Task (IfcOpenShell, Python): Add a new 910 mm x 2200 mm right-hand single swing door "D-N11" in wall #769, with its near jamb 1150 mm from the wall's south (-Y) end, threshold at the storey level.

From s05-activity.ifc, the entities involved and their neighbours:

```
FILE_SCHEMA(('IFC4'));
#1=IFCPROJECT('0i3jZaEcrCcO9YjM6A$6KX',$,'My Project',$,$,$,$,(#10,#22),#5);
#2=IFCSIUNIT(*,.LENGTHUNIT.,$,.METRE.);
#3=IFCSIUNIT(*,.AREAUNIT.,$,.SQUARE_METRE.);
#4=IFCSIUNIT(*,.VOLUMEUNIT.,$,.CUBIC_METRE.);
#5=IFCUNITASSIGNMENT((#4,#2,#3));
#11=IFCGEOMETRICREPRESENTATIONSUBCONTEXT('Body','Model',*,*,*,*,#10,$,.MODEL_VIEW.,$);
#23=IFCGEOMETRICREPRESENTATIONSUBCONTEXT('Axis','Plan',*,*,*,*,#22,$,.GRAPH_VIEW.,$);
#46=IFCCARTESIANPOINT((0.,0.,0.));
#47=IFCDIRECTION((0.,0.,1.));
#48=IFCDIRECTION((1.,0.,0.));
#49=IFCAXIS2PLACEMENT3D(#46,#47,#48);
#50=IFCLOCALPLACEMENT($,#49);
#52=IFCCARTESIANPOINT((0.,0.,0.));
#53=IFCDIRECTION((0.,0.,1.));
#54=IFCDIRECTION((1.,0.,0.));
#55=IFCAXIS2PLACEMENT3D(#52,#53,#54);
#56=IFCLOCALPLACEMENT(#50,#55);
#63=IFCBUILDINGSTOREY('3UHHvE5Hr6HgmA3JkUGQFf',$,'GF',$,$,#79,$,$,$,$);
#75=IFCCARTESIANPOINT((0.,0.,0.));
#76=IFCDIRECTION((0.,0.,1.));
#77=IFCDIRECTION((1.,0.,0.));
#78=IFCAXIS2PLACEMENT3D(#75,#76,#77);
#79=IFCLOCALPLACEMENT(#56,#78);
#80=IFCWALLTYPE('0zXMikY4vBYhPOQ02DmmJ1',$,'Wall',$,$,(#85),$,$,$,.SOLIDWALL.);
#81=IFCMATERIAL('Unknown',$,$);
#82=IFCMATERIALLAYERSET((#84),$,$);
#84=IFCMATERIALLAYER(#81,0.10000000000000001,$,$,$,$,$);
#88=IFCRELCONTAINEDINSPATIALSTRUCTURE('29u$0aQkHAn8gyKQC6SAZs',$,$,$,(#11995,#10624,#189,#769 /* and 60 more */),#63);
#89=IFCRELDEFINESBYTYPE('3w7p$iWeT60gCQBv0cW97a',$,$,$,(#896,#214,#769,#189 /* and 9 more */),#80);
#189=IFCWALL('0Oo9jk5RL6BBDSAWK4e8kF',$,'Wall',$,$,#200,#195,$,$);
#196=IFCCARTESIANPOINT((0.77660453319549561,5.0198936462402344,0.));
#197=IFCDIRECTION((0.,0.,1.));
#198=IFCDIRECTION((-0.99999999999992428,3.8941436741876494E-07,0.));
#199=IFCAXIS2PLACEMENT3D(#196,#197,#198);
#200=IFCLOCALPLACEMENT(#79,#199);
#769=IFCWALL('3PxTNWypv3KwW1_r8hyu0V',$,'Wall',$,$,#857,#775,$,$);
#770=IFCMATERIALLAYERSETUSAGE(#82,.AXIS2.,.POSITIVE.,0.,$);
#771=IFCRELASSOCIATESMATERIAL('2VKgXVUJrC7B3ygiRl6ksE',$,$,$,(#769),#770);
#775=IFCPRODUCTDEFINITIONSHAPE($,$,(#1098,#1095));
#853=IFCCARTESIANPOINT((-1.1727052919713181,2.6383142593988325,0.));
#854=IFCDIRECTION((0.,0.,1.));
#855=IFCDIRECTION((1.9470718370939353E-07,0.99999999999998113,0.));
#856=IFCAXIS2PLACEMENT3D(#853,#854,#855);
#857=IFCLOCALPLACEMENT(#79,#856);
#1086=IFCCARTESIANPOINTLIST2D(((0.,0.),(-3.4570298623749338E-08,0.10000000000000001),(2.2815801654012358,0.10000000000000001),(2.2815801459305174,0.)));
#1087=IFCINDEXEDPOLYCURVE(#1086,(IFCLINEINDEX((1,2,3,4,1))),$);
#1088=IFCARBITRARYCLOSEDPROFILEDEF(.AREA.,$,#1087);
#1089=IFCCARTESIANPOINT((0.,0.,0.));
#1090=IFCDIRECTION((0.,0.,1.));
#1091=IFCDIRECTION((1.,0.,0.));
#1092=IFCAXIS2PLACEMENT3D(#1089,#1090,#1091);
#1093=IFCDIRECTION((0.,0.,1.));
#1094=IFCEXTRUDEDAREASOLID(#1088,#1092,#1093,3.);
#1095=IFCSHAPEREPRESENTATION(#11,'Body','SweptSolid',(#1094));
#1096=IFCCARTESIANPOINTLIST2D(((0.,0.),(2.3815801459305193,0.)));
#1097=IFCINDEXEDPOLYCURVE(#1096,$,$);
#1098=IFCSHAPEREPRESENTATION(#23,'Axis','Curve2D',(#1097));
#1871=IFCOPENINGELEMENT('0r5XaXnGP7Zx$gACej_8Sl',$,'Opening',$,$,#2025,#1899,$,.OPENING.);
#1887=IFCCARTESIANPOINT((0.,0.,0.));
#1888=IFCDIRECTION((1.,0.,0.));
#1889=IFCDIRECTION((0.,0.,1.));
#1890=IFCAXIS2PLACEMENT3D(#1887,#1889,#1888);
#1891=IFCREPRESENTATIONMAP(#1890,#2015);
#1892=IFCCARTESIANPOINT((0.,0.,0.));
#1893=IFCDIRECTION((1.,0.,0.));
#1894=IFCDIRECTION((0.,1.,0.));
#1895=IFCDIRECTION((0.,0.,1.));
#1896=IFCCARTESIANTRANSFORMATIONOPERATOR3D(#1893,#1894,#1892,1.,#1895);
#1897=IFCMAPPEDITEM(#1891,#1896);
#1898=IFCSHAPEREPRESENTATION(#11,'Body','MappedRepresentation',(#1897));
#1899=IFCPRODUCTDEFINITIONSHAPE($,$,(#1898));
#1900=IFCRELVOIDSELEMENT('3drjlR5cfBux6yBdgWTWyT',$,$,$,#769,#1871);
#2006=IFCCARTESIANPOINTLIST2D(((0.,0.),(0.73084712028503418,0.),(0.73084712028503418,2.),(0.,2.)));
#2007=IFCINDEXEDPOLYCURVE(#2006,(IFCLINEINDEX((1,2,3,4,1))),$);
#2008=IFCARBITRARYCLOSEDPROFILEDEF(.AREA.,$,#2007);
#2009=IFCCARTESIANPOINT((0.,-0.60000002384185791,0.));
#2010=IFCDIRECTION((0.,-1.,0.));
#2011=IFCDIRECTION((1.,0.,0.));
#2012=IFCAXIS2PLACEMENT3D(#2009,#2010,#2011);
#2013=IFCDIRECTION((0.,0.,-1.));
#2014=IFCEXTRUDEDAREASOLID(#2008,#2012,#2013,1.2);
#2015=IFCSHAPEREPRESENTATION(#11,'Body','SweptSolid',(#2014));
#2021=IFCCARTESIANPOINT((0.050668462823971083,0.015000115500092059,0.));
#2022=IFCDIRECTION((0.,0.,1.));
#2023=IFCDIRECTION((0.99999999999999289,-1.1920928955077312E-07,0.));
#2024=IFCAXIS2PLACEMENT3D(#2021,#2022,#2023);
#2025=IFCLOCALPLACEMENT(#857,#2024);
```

```python
import numpy as np
import ifcopenshell
import ifcopenshell.api.feature
import ifcopenshell.api.geometry
import ifcopenshell.api.root
import ifcopenshell.api.spatial
import ifcopenshell.geom
import ifcopenshell.util.element
import ifcopenshell.util.placement
import ifcopenshell.util.representation
import ifcopenshell.util.shape
import ifcopenshell.util.unit

model = ifcopenshell.open("s05-activity.ifc")
unit_scale = ifcopenshell.util.unit.calculate_unit_scale(model)
settings = ifcopenshell.geom.settings()


def volume(element):
    """Net volume in cubic metres, openings subtracted."""
    shape = ifcopenshell.geom.create_shape(settings, element)
    return ifcopenshell.util.shape.get_volume(shape.geometry)


wall = model.by_id(769)
storey = ifcopenshell.util.element.get_container(wall, ifc_class="IfcBuildingStorey")
context = ifcopenshell.util.representation.get_context(model, "Model", "Body", "MODEL_VIEW")
before = volume(wall)

width, height, from_end, sill = 0.91, 2.2, 1.15, 0.0  # metres

# The wall runs along its own X axis, and the end named is its -X end.
wall_shape = ifcopenshell.geom.create_shape(settings, wall)
x, y, z = ifcopenshell.util.shape.get_vertices(wall_shape.geometry).T
start = x.min() + from_end
face, thickness = float(y.min()), float(y.max() - y.min())
wall_matrix = ifcopenshell.util.placement.get_local_placement(wall.ObjectPlacement)
level = ifcopenshell.util.placement.get_local_placement(storey.ObjectPlacement)[2, 3]


def in_wall(x, y):
    """Placement at x, y metres in the wall's axes, at sill height."""
    matrix = wall_matrix.copy()
    matrix[:, 3] = wall_matrix @ np.array([x / unit_scale, y / unit_scale, 0.0, 1.0])
    matrix[2, 3] = level + sill / unit_scale
    return matrix


# Opening: a box that overshoots both wall faces by 50 mm.
opening = ifcopenshell.api.root.create_entity(model, ifc_class="IfcOpeningElement", predefined_type="OPENING")
box = ifcopenshell.api.geometry.add_wall_representation(
    model, context=context, length=width, height=height, thickness=thickness + 0.1
)
ifcopenshell.api.geometry.assign_representation(model, product=opening, representation=box)
ifcopenshell.api.geometry.edit_object_placement(model, product=opening, matrix=in_wall(start, face - 0.05), is_si=False)
ifcopenshell.api.feature.add_feature(model, feature=opening, element=wall)

door = ifcopenshell.api.root.create_entity(model, ifc_class="IfcDoor", name="D-N11", predefined_type="DOOR")
door.OverallWidth, door.OverallHeight = width / unit_scale, height / unit_scale
door.OperationType = "SINGLE_SWING_RIGHT"
body = ifcopenshell.api.geometry.add_door_representation(
    model,
    context=context,
    overall_width=door.OverallWidth,
    overall_height=door.OverallHeight,
    operation_type="SINGLE_SWING_RIGHT",
    lining_properties={"LiningDepth": thickness / unit_scale, "ThresholdDepth": thickness / unit_scale},
)
ifcopenshell.api.geometry.assign_representation(model, product=door, representation=body)
ifcopenshell.api.spatial.assign_container(model, products=[door], relating_structure=storey)
ifcopenshell.api.feature.add_filling(model, opening=opening, element=door)

# The lining spans the wall, so the door starts at the wall face.
ifcopenshell.api.geometry.edit_object_placement(model, product=door, matrix=in_wall(start, face), is_si=False)

after = volume(wall)

print(f"wall volume {before:.3f} -> {after:.3f} m3")

model.write("s05-activity_updated.ifc")
```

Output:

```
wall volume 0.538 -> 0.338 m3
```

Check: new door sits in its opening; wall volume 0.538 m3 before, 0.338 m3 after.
